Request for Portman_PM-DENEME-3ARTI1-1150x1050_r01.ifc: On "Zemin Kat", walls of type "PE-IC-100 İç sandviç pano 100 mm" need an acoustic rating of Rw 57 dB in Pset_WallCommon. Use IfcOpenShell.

First a look at what the model holds.

```python
import ifcopenshell
import ifcopenshell.util.element

model = ifcopenshell.open("Portman_PM-DENEME-3ARTI1-1150x1050_r01.ifc")
print(model.schema)
storey = next(s for s in model.by_type("IfcBuildingStorey") if s.Name == "Zemin Kat")
walls = [e for e in ifcopenshell.util.element.get_decomposition(storey) if e.is_a("IfcWall")]
seen = {}
for e in walls:
    element_type = ifcopenshell.util.element.get_type(e)
    key = (element_type.Name if element_type != e and element_type else None, ifcopenshell.util.element.get_pset(e, "Pset_WallCommon", "AcousticRating"))
    seen[key] = seen.get(key, 0) + 1
for (name, value), count in sorted(seen.items(), key=str):
    print(count, "x", name, "|", value)
```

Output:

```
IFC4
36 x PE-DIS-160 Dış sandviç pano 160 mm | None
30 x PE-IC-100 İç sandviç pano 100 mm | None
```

```python
import ifcopenshell
import ifcopenshell.api.pset
import ifcopenshell.util.element

model = ifcopenshell.open("Portman_PM-DENEME-3ARTI1-1150x1050_r01.ifc")

storey = next(s for s in model.by_type("IfcBuildingStorey") if s.Name == "Zemin Kat")
walls = [e for e in ifcopenshell.util.element.get_decomposition(storey) if e.is_a("IfcWall")]

count = 0
for e in walls:
    element_type = ifcopenshell.util.element.get_type(e)
    if element_type in (None, e) or element_type.Name != "PE-IC-100 İç sandviç pano 100 mm":
        continue
    # add_pset returns the element's existing set when there is one.
    pset = ifcopenshell.api.pset.add_pset(model, product=e, name="Pset_WallCommon")
    ifcopenshell.api.pset.edit_pset(model, pset=pset, properties={"AcousticRating": "Rw 57 dB"})
    count += 1

print(count, "walls updated")

model.write("Portman_PM-DENEME-3ARTI1-1150x1050_r01-out.ifc")
```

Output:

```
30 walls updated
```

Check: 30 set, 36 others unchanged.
